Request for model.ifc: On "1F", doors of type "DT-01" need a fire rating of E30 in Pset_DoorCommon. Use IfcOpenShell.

First a look at what the model holds.

```python
import ifcopenshell
import ifcopenshell.util.element

model = ifcopenshell.open("model.ifc")
print(model.schema)
storey = next(s for s in model.by_type("IfcBuildingStorey") if s.Name == "1F")
doors = [e for e in ifcopenshell.util.element.get_decomposition(storey) if e.is_a("IfcDoor")]
seen = {}
for e in doors:
    element_type = ifcopenshell.util.element.get_type(e)
    key = (element_type.Name if element_type != e and element_type else None, ifcopenshell.util.element.get_pset(e, "Pset_DoorCommon", "FireRating"))
    seen[key] = seen.get(key, 0) + 1
for (name, value), count in sorted(seen.items(), key=str):
    print(count, "x", name, "|", value)
```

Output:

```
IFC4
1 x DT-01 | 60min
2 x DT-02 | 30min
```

```python
import ifcopenshell
import ifcopenshell.api.pset
import ifcopenshell.util.element

model = ifcopenshell.open("model.ifc")

storey = next(s for s in model.by_type("IfcBuildingStorey") if s.Name == "1F")
doors = [e for e in ifcopenshell.util.element.get_decomposition(storey) if e.is_a("IfcDoor")]

count = 0
for e in doors:
    element_type = ifcopenshell.util.element.get_type(e)
    if element_type in (None, e) or element_type.Name != "DT-01":
        continue
    # add_pset returns the element's existing set when there is one.
    pset = ifcopenshell.api.pset.add_pset(model, product=e, name="Pset_DoorCommon")
    ifcopenshell.api.pset.edit_pset(model, pset=pset, properties={"FireRating": "E30"})
    count += 1

print(count, "doors updated")

model.write("model_edited.ifc")
```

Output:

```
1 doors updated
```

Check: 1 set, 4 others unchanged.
